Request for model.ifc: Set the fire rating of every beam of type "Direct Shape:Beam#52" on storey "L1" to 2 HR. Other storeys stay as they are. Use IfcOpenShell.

First a look at what the model holds.

```python
import ifcopenshell
import ifcopenshell.util.element

model = ifcopenshell.open("model.ifc")
print(model.schema)
storey = next(s for s in model.by_type("IfcBuildingStorey") if s.Name == "L1")
beams = [e for e in ifcopenshell.util.element.get_decomposition(storey) if e.is_a("IfcBeam")]
seen = {}
for e in beams:
    element_type = ifcopenshell.util.element.get_type(e)
    key = (element_type.Name if element_type != e and element_type else None, ifcopenshell.util.element.get_pset(e, "Pset_BeamCommon", "FireRating"))
    seen[key] = seen.get(key, 0) + 1
for (name, value), count in sorted(seen.items(), key=str):
    print(count, "x", name, "|", value)
```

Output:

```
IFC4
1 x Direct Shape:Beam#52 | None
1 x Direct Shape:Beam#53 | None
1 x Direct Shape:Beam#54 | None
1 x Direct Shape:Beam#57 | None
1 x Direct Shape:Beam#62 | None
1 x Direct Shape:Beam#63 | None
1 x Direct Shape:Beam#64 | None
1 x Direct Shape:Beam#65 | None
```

```python
import ifcopenshell
import ifcopenshell.api.pset
import ifcopenshell.util.element

model = ifcopenshell.open("model.ifc")

storey = next(s for s in model.by_type("IfcBuildingStorey") if s.Name == "L1")
beams = [e for e in ifcopenshell.util.element.get_decomposition(storey) if e.is_a("IfcBeam")]

count = 0
for e in beams:
    element_type = ifcopenshell.util.element.get_type(e)
    if element_type in (None, e) or element_type.Name != "Direct Shape:Beam#52":
        continue
    # add_pset returns the element's existing set when there is one.
    pset = ifcopenshell.api.pset.add_pset(model, product=e, name="Pset_BeamCommon")
    ifcopenshell.api.pset.edit_pset(model, pset=pset, properties={"FireRating": "2 HR"})
    count += 1

print(count, "beams updated")

model.write("model_updated.ifc")
```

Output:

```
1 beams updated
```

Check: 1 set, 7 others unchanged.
